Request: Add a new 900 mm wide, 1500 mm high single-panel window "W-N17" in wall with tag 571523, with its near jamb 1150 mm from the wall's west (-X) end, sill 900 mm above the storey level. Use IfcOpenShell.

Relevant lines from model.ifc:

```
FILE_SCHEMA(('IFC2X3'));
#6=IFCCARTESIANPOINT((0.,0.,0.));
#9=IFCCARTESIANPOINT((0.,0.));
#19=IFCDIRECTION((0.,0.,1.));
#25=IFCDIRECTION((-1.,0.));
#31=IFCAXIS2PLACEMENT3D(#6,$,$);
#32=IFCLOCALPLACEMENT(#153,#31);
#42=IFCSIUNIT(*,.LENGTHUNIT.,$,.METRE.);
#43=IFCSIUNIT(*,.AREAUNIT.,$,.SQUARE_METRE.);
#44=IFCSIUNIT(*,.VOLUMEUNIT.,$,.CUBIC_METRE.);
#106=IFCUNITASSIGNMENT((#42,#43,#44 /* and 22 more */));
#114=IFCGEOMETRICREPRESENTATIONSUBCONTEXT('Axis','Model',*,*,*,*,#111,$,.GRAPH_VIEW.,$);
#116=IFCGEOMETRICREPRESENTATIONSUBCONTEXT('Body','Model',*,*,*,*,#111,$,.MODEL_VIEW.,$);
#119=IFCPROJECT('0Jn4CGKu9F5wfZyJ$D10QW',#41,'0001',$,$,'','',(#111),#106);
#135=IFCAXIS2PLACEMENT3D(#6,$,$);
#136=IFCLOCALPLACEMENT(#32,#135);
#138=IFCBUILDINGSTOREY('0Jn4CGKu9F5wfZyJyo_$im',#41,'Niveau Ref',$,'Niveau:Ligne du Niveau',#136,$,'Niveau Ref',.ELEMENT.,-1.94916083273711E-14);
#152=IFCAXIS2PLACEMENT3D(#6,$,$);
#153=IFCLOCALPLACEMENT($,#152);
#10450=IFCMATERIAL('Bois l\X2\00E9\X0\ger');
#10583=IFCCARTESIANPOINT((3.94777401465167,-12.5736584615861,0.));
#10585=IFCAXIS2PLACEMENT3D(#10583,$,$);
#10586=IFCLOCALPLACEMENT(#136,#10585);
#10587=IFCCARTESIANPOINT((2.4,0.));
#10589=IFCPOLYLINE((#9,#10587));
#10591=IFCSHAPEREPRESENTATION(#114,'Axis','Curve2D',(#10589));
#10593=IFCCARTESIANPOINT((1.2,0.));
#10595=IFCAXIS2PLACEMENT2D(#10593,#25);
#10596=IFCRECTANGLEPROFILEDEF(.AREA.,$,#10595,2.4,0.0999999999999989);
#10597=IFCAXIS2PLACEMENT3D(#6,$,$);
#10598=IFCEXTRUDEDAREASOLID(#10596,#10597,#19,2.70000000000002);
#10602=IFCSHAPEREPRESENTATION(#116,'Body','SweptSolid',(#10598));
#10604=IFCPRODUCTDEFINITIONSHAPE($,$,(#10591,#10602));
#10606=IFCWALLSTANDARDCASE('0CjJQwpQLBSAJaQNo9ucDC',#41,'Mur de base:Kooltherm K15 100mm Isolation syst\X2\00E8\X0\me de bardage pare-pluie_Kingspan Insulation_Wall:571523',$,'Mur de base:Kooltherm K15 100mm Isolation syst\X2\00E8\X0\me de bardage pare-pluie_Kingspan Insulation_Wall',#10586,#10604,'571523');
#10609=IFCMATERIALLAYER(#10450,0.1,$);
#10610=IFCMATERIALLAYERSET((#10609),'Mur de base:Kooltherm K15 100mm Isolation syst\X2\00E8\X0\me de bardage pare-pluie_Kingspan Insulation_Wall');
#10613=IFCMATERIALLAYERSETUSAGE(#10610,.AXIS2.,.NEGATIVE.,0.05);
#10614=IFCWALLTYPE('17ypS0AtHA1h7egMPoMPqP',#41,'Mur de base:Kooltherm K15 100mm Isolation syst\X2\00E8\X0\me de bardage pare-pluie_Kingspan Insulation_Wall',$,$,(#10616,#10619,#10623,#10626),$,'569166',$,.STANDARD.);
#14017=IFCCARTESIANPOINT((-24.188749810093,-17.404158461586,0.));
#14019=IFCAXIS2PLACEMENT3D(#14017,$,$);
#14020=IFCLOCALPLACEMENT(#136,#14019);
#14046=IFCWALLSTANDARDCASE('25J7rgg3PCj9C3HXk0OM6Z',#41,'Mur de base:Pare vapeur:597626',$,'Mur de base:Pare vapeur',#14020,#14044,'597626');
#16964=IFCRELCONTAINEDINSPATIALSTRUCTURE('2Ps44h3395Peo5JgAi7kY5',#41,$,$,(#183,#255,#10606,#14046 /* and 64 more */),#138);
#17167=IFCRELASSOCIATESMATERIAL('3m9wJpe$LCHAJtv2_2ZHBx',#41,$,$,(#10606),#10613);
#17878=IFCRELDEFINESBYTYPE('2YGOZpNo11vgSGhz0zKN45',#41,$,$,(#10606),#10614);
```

```python
import numpy as np
import ifcopenshell
import ifcopenshell.api.feature
import ifcopenshell.api.geometry
import ifcopenshell.api.root
import ifcopenshell.api.spatial
import ifcopenshell.api.type
import ifcopenshell.geom
import ifcopenshell.util.element
import ifcopenshell.util.placement
import ifcopenshell.util.representation
import ifcopenshell.util.shape
import ifcopenshell.util.unit

model = ifcopenshell.open("model.ifc")
unit_scale = ifcopenshell.util.unit.calculate_unit_scale(model)
settings = ifcopenshell.geom.settings()


def volume(element):
    """Net volume in cubic metres, openings subtracted."""
    shape = ifcopenshell.geom.create_shape(settings, element)
    return ifcopenshell.util.shape.get_volume(shape.geometry)


wall = model.by_guid("0CjJQwpQLBSAJaQNo9ucDC")
storey = ifcopenshell.util.element.get_container(wall, ifc_class="IfcBuildingStorey")
context = ifcopenshell.util.representation.get_context(model, "Model", "Body", "MODEL_VIEW")
before = volume(wall)

width, height, from_end, sill = 0.9, 1.5, 1.15, 0.9  # metres

# The wall runs along its own X axis, and the end named is its -X end.
wall_shape = ifcopenshell.geom.create_shape(settings, wall)
x, y, z = ifcopenshell.util.shape.get_vertices(wall_shape.geometry).T
start = x.min() + from_end
face, thickness = float(y.min()), float(y.max() - y.min())
wall_matrix = ifcopenshell.util.placement.get_local_placement(wall.ObjectPlacement)
level = ifcopenshell.util.placement.get_local_placement(storey.ObjectPlacement)[2, 3]


def in_wall(x, y):
    """Placement at x, y metres in the wall's axes, at sill height."""
    matrix = wall_matrix.copy()
    matrix[:, 3] = wall_matrix @ np.array([x / unit_scale, y / unit_scale, 0.0, 1.0])
    matrix[2, 3] = level + sill / unit_scale
    return matrix


# Opening: a box that overshoots both wall faces by 50 mm.
opening = ifcopenshell.api.root.create_entity(model, ifc_class="IfcOpeningElement")
box = ifcopenshell.api.geometry.add_wall_representation(
    model, context=context, length=width, height=height, thickness=thickness + 0.1
)
ifcopenshell.api.geometry.assign_representation(model, product=opening, representation=box)
ifcopenshell.api.geometry.edit_object_placement(model, product=opening, matrix=in_wall(start, face - 0.05), is_si=False)
ifcopenshell.api.feature.add_feature(model, feature=opening, element=wall)

window = ifcopenshell.api.root.create_entity(model, ifc_class="IfcWindow", name="W-N17")
window.OverallWidth, window.OverallHeight = width / unit_scale, height / unit_scale
body = ifcopenshell.api.geometry.add_window_representation(
    model,
    context=context,
    overall_width=window.OverallWidth,
    overall_height=window.OverallHeight,
    partition_type="SINGLE_PANEL",
)
ifcopenshell.api.geometry.assign_representation(model, product=window, representation=body)
ifcopenshell.api.spatial.assign_container(model, products=[window], relating_structure=storey)
fills = ifcopenshell.api.feature.add_filling(model, opening=opening, element=window)
fills.OwnerHistory = window.OwnerHistory  # required in IFC2X3

# IFC2X3 keeps the operation on the window style.
style = ifcopenshell.api.root.create_entity(model, ifc_class="IfcWindowStyle", name="W-N17")
style.OperationType, style.ConstructionType = "SINGLE_PANEL", "NOTDEFINED"
style.ParameterTakesPrecedence = style.Sizeable = False
ifcopenshell.api.type.assign_type(model, related_objects=[window], relating_type=style)

# Centre the window in the wall's thickness.
ifcopenshell.api.geometry.edit_object_placement(model, product=window, matrix=in_wall(start, face), is_si=False)
window_shape = ifcopenshell.geom.create_shape(settings, window)
depth = ifcopenshell.util.shape.get_vertices(window_shape.geometry)[:, 1]
offset = face + thickness / 2 - (depth.min() + depth.max()) / 2
ifcopenshell.api.geometry.edit_object_placement(model, product=window, matrix=in_wall(start, offset), is_si=False)

after = volume(wall)

print(f"wall volume {before:.3f} -> {after:.3f} m3")

model.write("model_rev.ifc")
```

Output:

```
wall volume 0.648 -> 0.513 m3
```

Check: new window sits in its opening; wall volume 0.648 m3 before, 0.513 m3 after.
